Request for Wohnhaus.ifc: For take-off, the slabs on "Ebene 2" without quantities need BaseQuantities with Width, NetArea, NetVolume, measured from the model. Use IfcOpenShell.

First a look at what the model holds.

```python
import ifcopenshell
import ifcopenshell.util.element
import ifcopenshell.util.unit

model = ifcopenshell.open("Wohnhaus.ifc")
print(model.schema)
for unit_type in ("LENGTHUNIT", "AREAUNIT", "VOLUMEUNIT"):
    print(unit_type, ifcopenshell.util.unit.calculate_unit_scale(model, unit_type))
storey = next(s for s in model.by_type("IfcBuildingStorey") if s.Name == "Ebene 2")
slabs = [e for e in ifcopenshell.util.element.get_decomposition(storey) if e.is_a("IfcSlab")]
for e in sorted(slabs, key=lambda e: e.id()):
    print(e.id(), e.is_a(), e.Name, list(ifcopenshell.util.element.get_psets(e, qtos_only=True)), sep=" | ")
```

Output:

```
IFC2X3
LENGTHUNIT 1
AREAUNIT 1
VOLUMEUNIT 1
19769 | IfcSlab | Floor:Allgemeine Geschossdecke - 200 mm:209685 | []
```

```python
import ifcopenshell
import ifcopenshell.api.pset
import ifcopenshell.geom
import ifcopenshell.util.element
import ifcopenshell.util.shape
import ifcopenshell.util.unit

model = ifcopenshell.open("Wohnhaus.ifc")
unit_scale = ifcopenshell.util.unit.calculate_unit_scale(model)
area_scale = ifcopenshell.util.unit.calculate_unit_scale(model, "AREAUNIT")
volume_scale = ifcopenshell.util.unit.calculate_unit_scale(model, "VOLUMEUNIT")
settings = ifcopenshell.geom.settings()

storey = next(s for s in model.by_type("IfcBuildingStorey") if s.Name == "Ebene 2")
slabs = [e for e in ifcopenshell.util.element.get_decomposition(storey) if e.is_a("IfcSlab")]

for e in sorted(slabs, key=lambda e: e.id()):
    if ifcopenshell.util.element.get_psets(e, qtos_only=True, should_inherit=False):
        continue
    # Geometry comes back in metres, in the element's own axes.
    shape = ifcopenshell.geom.create_shape(settings, e)
    values = {
        "Width": ifcopenshell.util.shape.get_z(shape.geometry) / unit_scale,
        "NetArea": ifcopenshell.util.shape.get_footprint_area(shape.geometry) / area_scale,
        "NetVolume": ifcopenshell.util.shape.get_volume(shape.geometry) / volume_scale,
    }
    qto = ifcopenshell.api.pset.add_qto(model, product=e, name="BaseQuantities")
    ifcopenshell.api.pset.edit_qto(model, qto=qto, properties=values)
    print(e.id(), {k: round(v, 3) for k, v in values.items()})

model.write("Wohnhaus_edited.ifc")
```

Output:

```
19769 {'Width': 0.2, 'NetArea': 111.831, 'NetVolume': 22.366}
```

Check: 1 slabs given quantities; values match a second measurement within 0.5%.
